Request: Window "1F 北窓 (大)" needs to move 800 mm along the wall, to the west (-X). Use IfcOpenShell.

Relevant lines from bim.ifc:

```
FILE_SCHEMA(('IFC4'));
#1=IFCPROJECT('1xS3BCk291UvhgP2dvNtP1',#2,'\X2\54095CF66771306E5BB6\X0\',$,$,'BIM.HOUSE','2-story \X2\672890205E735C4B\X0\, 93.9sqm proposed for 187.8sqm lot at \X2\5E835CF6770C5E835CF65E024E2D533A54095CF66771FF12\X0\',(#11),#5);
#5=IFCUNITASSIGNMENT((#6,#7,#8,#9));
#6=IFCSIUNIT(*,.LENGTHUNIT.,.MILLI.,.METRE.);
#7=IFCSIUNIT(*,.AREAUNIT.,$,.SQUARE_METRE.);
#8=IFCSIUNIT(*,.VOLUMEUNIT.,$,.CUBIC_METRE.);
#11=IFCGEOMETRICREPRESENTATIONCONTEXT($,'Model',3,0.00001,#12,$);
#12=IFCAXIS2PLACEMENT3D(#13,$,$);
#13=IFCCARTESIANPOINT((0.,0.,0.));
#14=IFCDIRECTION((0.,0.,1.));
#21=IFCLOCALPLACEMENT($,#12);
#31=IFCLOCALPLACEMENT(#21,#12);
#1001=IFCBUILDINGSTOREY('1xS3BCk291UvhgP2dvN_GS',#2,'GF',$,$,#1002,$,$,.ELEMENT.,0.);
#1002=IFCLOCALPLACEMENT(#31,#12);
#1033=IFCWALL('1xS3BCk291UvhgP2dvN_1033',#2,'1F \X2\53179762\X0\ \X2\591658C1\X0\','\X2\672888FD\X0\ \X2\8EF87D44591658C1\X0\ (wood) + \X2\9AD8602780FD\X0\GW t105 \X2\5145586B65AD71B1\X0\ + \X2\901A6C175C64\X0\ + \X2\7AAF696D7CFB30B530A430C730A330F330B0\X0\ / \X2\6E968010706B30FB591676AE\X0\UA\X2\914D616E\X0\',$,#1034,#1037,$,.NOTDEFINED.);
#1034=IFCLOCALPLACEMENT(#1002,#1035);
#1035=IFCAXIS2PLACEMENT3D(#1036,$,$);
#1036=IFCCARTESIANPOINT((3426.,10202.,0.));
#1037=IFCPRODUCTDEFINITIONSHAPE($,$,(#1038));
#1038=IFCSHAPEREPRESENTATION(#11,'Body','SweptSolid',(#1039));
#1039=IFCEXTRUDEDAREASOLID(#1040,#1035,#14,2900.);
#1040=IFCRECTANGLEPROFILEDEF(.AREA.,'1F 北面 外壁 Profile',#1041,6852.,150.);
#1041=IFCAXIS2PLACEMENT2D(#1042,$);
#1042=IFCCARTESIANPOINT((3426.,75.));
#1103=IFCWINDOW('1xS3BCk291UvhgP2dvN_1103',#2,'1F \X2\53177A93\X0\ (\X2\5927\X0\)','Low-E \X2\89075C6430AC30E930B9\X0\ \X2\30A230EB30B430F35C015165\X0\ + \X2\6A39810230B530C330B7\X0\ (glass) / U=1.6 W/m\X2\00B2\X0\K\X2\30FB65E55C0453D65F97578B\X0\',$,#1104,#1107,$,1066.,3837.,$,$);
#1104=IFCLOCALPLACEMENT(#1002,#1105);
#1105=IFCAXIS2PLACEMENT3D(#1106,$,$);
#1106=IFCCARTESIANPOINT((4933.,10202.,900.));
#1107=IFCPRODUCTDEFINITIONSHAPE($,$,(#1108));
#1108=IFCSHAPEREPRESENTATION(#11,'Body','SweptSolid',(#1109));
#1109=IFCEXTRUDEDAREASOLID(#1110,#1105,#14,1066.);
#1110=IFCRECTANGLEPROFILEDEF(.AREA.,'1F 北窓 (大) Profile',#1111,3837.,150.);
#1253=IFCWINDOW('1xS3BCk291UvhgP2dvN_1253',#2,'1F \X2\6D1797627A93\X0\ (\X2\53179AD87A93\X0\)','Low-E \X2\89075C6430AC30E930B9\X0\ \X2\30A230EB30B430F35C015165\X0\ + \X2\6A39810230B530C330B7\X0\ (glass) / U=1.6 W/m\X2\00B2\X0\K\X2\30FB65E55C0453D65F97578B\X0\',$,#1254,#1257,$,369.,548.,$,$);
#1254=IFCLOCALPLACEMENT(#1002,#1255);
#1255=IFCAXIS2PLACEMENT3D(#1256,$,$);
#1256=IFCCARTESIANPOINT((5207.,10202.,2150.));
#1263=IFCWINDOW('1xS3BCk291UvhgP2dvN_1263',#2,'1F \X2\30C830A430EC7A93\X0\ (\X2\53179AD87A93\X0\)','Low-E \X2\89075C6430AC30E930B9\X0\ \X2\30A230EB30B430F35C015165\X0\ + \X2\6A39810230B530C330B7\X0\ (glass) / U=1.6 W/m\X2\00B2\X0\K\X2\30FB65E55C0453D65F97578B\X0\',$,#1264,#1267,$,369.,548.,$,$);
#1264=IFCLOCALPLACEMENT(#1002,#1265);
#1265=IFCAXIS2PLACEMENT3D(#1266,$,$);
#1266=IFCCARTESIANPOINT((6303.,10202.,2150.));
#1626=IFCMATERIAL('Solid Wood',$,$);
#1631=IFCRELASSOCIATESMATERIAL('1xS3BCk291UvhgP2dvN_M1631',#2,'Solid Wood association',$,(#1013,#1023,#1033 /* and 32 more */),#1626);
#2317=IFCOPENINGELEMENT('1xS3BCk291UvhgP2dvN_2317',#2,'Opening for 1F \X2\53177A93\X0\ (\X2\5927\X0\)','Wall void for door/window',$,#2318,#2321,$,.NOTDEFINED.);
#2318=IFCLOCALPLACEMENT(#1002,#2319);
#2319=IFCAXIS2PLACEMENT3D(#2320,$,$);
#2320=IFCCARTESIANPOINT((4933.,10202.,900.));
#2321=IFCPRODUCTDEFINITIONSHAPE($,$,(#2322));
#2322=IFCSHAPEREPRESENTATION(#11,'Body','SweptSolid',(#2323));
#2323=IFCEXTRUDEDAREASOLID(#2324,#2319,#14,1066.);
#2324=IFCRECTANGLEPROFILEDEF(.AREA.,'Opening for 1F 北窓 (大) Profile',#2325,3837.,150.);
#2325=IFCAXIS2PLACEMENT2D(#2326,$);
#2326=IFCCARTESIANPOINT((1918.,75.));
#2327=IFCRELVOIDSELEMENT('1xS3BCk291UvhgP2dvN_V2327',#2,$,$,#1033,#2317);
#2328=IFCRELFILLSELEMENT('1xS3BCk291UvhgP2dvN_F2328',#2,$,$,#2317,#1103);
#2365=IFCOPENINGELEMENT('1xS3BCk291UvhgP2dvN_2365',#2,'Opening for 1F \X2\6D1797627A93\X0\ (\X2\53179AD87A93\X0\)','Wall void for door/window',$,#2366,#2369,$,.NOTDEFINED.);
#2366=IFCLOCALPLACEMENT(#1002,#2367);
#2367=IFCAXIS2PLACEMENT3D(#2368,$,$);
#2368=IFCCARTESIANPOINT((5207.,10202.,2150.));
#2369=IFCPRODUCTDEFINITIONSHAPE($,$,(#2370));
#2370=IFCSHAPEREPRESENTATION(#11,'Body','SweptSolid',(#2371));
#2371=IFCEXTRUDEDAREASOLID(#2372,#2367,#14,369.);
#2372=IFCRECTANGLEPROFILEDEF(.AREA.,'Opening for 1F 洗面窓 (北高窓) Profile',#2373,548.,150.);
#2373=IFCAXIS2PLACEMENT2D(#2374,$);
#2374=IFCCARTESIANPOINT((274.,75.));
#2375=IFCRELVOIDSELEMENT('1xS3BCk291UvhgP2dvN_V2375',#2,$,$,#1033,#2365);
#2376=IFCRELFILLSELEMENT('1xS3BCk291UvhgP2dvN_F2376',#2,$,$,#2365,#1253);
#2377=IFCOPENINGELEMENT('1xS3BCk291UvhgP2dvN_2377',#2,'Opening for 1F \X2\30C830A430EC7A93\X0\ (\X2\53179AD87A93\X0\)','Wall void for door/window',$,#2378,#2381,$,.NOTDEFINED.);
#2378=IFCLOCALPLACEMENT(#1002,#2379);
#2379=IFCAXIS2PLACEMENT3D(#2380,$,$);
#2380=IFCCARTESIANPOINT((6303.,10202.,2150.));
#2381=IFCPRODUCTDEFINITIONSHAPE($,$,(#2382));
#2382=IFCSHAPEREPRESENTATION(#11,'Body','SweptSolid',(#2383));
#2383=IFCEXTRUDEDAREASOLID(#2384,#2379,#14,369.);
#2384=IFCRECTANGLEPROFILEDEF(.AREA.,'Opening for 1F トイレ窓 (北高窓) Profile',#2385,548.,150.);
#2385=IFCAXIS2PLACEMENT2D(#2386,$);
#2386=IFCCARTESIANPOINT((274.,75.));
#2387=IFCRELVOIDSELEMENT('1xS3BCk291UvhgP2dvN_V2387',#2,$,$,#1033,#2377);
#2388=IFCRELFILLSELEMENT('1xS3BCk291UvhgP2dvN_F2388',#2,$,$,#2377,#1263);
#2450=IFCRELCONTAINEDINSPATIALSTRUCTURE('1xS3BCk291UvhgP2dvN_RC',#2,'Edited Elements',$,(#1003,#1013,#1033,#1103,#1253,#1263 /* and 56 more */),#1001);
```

```python
import ifcopenshell
import ifcopenshell.api.geometry
import ifcopenshell.util.placement

model = ifcopenshell.open("bim.ifc")

window = model.by_guid("1xS3BCk291UvhgP2dvN_1103")
opening = window.FillsVoids[0].RelatingOpeningElement
wall = opening.VoidsElements[0].RelatingBuildingElement

wall_matrix = ifcopenshell.util.placement.get_local_placement(wall.ObjectPlacement)
shift = wall_matrix[:3, 0] * -800.0
before = ifcopenshell.util.placement.get_local_placement(window.ObjectPlacement)[:3, 3].copy()

# The window is not placed relative to its opening, so move both.
for product in (opening, window):
    matrix = ifcopenshell.util.placement.get_local_placement(product.ObjectPlacement)
    matrix[:3, 3] += shift
    ifcopenshell.api.geometry.edit_object_placement(model, product=product, matrix=matrix, is_si=False)

after = ifcopenshell.util.placement.get_local_placement(window.ObjectPlacement)[:3, 3]
print("window moved by", (after - before).round(3) + 0.0)

model.write("bim_updated.ifc")
```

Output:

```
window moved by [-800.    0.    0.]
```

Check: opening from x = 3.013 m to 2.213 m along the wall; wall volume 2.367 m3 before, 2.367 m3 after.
